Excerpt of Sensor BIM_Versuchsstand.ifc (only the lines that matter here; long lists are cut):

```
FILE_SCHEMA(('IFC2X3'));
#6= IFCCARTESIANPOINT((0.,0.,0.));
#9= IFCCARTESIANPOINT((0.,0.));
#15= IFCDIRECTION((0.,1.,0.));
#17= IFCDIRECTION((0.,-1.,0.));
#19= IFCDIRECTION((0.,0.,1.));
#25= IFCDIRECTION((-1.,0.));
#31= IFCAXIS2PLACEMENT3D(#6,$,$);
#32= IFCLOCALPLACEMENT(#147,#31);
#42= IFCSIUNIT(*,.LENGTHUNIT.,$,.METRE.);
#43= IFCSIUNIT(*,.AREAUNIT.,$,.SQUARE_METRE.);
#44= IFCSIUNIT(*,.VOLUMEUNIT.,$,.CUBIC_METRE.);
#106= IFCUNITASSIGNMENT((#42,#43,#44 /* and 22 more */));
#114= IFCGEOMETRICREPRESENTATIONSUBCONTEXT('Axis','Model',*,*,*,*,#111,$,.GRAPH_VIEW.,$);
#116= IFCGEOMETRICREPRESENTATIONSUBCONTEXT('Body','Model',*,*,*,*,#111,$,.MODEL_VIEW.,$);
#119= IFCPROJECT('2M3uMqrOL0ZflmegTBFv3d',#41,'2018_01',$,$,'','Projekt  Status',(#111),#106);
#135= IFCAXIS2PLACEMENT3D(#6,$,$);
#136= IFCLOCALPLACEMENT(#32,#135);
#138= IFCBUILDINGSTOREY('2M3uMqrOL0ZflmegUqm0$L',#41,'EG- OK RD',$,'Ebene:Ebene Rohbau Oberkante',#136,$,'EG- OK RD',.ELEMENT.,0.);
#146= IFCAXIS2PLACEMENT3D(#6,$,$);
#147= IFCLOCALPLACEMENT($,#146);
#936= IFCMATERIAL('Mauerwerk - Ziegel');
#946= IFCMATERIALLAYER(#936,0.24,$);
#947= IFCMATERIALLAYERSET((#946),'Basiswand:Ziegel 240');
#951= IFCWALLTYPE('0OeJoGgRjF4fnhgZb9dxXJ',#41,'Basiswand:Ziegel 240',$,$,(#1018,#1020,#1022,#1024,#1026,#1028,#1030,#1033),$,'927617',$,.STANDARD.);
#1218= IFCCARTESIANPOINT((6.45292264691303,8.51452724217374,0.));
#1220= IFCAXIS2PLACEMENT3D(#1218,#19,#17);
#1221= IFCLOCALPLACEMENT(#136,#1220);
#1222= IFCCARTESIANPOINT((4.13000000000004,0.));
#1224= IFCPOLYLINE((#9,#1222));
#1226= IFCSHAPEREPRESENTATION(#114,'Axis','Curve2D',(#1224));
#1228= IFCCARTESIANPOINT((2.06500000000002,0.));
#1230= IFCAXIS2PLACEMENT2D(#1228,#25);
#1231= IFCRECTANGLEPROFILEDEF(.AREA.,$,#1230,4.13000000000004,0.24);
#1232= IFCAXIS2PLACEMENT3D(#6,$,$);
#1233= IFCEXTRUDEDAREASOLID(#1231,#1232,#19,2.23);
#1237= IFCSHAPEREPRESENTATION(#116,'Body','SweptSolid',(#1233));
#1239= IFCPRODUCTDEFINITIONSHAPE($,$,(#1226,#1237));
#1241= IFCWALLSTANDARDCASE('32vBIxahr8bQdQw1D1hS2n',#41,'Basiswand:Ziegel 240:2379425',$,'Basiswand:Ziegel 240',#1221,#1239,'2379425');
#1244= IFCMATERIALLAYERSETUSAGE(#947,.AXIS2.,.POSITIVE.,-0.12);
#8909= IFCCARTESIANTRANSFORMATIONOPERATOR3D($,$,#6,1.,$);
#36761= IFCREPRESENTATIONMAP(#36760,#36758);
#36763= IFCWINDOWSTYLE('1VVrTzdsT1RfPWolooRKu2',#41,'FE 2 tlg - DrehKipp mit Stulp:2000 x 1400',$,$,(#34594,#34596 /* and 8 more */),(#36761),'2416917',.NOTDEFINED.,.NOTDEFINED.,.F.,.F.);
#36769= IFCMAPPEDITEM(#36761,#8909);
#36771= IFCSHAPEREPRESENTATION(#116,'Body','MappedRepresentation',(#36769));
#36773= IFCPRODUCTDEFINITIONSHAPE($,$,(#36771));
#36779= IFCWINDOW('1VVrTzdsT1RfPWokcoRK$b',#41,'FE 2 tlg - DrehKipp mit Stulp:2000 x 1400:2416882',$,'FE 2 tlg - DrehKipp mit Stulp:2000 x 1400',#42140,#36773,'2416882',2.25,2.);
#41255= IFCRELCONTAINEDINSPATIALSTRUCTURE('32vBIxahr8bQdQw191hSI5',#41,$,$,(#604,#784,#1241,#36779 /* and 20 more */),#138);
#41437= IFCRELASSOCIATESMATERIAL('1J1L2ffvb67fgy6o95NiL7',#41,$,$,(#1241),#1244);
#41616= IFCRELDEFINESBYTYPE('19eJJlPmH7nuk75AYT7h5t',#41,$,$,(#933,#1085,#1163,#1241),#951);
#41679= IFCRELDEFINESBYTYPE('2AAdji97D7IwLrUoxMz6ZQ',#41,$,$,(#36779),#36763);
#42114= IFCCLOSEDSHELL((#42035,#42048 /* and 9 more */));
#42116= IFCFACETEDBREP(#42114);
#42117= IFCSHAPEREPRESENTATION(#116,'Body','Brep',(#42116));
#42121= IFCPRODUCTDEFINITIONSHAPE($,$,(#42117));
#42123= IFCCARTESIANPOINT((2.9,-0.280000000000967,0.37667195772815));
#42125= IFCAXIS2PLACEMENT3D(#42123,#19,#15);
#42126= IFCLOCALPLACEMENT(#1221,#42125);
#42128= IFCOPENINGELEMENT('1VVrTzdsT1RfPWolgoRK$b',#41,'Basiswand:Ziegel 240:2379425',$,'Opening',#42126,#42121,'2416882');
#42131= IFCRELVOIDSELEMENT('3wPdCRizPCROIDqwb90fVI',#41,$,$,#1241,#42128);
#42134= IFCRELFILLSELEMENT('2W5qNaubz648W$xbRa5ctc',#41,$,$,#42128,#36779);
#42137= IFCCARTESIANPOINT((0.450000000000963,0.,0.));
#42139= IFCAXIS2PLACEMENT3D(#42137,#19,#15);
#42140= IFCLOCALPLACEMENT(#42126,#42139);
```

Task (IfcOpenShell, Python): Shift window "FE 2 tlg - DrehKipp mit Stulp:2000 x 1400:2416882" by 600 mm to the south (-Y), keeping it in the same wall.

```python
import ifcopenshell
import ifcopenshell.api.geometry
import ifcopenshell.util.placement

model = ifcopenshell.open("Sensor BIM_Versuchsstand.ifc")

window = model.by_guid("1VVrTzdsT1RfPWokcoRK$b")
opening = window.FillsVoids[0].RelatingOpeningElement
wall = opening.VoidsElements[0].RelatingBuildingElement

wall_matrix = ifcopenshell.util.placement.get_local_placement(wall.ObjectPlacement)
shift = wall_matrix[:3, 0] * 0.6
before = ifcopenshell.util.placement.get_local_placement(window.ObjectPlacement)[:3, 3].copy()

# The window is placed relative to its opening, so it follows when the opening moves.
matrix = ifcopenshell.util.placement.get_local_placement(opening.ObjectPlacement)
matrix[:3, 3] += shift
ifcopenshell.api.geometry.edit_object_placement(
    model, product=opening, matrix=matrix, is_si=False, should_transform_children=True
)

after = ifcopenshell.util.placement.get_local_placement(window.ObjectPlacement)[:3, 3]
print("window moved by", (after - before).round(3) + 0.0)

model.write("Sensor BIM_Versuchsstand_rev.ifc")
```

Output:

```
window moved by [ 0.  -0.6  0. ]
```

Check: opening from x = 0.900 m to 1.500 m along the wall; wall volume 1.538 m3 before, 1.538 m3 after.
